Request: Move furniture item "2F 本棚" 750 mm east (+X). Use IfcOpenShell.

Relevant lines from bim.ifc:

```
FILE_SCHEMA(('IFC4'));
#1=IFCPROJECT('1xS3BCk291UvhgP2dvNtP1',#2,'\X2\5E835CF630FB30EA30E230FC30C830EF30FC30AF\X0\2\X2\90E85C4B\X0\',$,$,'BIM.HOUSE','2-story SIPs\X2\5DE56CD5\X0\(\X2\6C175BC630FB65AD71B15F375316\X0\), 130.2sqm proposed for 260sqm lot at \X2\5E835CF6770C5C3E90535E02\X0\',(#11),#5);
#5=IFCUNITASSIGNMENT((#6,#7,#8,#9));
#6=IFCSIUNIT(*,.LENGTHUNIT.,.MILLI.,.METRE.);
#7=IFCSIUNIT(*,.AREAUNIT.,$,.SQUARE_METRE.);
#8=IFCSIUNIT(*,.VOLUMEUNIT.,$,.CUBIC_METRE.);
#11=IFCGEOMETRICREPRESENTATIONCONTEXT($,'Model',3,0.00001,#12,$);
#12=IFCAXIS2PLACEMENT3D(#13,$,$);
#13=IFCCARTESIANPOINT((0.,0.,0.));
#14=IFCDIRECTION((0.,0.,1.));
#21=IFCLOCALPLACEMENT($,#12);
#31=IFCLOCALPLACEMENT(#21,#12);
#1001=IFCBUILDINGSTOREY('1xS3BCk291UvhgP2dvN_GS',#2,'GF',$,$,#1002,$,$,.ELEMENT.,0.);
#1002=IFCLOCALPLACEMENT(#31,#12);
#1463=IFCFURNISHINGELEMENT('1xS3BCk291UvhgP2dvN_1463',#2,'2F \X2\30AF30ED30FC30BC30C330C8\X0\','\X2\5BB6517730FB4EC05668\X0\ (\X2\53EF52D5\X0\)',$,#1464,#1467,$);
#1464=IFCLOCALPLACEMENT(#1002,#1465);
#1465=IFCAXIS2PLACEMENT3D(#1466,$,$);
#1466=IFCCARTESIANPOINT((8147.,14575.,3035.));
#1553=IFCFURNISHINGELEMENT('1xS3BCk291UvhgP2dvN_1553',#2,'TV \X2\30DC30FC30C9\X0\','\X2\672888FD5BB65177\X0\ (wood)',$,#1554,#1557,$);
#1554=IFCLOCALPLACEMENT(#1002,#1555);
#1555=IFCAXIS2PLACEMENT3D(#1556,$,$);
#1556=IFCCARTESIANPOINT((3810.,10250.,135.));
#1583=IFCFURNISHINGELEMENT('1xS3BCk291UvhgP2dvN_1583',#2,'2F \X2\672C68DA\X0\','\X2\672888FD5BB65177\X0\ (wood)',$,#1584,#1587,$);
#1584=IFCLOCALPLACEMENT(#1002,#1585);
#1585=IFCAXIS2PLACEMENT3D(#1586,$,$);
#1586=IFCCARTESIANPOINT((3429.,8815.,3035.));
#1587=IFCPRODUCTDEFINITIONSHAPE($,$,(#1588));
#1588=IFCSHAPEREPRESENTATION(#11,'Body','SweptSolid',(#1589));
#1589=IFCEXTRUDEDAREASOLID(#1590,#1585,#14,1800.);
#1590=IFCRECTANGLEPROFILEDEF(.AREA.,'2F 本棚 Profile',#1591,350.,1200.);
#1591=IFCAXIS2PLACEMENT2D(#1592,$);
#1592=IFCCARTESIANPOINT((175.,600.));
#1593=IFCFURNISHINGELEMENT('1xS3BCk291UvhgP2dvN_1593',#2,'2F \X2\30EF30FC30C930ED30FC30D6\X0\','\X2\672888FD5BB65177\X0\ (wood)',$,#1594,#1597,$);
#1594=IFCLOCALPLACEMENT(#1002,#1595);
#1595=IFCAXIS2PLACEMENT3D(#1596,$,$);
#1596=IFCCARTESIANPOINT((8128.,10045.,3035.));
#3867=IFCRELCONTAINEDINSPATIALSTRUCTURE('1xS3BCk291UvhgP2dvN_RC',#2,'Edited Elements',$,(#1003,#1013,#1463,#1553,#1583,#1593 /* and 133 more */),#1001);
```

```python
import ifcopenshell
import ifcopenshell.api.geometry
import ifcopenshell.util.placement

model = ifcopenshell.open("bim.ifc")

item = model.by_guid("1xS3BCk291UvhgP2dvN_1583")
matrix = ifcopenshell.util.placement.get_local_placement(item.ObjectPlacement)
matrix[0, 3] += 750.0
ifcopenshell.api.geometry.edit_object_placement(model, product=item, matrix=matrix, is_si=False)

print(ifcopenshell.util.placement.get_local_placement(item.ObjectPlacement).round(3) + 0.0)

model.write("bim_v2.ifc")
```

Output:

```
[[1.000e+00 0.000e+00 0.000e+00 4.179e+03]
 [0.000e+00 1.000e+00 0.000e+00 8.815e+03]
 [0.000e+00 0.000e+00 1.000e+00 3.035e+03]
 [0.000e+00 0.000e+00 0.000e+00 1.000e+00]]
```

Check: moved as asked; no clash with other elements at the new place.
